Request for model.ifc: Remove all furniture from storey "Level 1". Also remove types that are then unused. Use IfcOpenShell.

First a look at what the model holds.

```python
import ifcopenshell
import ifcopenshell.util.element

model = ifcopenshell.open("model.ifc")
print(model.schema)
storey = next(s for s in model.by_type("IfcBuildingStorey") if s.Name == "Level 1")
furniture = [e for e in ifcopenshell.util.element.get_decomposition(storey) if e.is_a("IfcFurnishingElement")]
seen = {}
for e in furniture:
    element_type = ifcopenshell.util.element.get_type(e)
    name = element_type.Name if element_type not in (None, e) else None
    seen[name] = seen.get(name, 0) + 1
for name, count in sorted(seen.items(), key=str):
    print(count, "x", name)
```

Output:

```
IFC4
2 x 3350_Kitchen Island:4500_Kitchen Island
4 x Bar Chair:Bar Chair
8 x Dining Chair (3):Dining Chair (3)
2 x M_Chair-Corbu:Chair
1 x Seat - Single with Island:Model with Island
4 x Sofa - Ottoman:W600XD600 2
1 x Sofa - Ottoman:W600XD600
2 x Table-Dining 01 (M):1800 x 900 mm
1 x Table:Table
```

```python
import ifcopenshell
import ifcopenshell.api.root
import ifcopenshell.util.element

model = ifcopenshell.open("model.ifc")

storey = next(s for s in model.by_type("IfcBuildingStorey") if s.Name == "Level 1")
furniture = [e for e in ifcopenshell.util.element.get_decomposition(storey) if e.is_a("IfcFurnishingElement")]
types = {ifcopenshell.util.element.get_type(e) for e in furniture} - {None, *furniture}

for e in furniture:
    ifcopenshell.api.root.remove_product(model, product=e)
print(len(furniture), "removed")

unused = [t for t in types if not ifcopenshell.util.element.get_types(t)]
for t in unused:
    ifcopenshell.api.root.remove_product(model, product=t)
print(len(unused), "unused types removed")

model.write("model_edited.ifc")
```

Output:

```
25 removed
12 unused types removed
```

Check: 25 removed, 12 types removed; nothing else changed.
